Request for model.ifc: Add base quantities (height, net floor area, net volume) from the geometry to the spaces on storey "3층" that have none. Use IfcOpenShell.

First a look at what the model holds.

```python
import ifcopenshell
import ifcopenshell.util.element
import ifcopenshell.util.unit

model = ifcopenshell.open("model.ifc")
print(model.schema)
for unit_type in ("LENGTHUNIT", "AREAUNIT", "VOLUMEUNIT"):
    print(unit_type, ifcopenshell.util.unit.calculate_unit_scale(model, unit_type))
storey = next(s for s in model.by_type("IfcBuildingStorey") if s.Name == "3층")
spaces = [e for e in ifcopenshell.util.element.get_decomposition(storey) if e.is_a("IfcSpace")]
for e in sorted(spaces, key=lambda e: e.id()):
    print(e.id(), e.is_a(), e.Name, list(ifcopenshell.util.element.get_psets(e, qtos_only=True)), sep=" | ")
```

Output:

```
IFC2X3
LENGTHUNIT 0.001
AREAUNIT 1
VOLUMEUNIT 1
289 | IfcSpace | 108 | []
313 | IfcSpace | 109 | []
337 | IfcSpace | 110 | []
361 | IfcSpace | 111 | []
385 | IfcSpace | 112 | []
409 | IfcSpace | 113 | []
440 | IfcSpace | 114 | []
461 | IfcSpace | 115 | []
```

```python
import ifcopenshell
import ifcopenshell.api.pset
import ifcopenshell.geom
import ifcopenshell.util.element
import ifcopenshell.util.shape
import ifcopenshell.util.unit

model = ifcopenshell.open("model.ifc")
unit_scale = ifcopenshell.util.unit.calculate_unit_scale(model)
area_scale = ifcopenshell.util.unit.calculate_unit_scale(model, "AREAUNIT")
volume_scale = ifcopenshell.util.unit.calculate_unit_scale(model, "VOLUMEUNIT")
settings = ifcopenshell.geom.settings()

storey = next(s for s in model.by_type("IfcBuildingStorey") if s.Name == "3층")
spaces = [e for e in ifcopenshell.util.element.get_decomposition(storey) if e.is_a("IfcSpace")]

for e in sorted(spaces, key=lambda e: e.id()):
    if ifcopenshell.util.element.get_psets(e, qtos_only=True, should_inherit=False):
        continue
    # Geometry comes back in metres, in the element's own axes.
    shape = ifcopenshell.geom.create_shape(settings, e)
    values = {
        "Height": ifcopenshell.util.shape.get_z(shape.geometry) / unit_scale,
        "NetFloorArea": ifcopenshell.util.shape.get_footprint_area(shape.geometry) / area_scale,
        "NetVolume": ifcopenshell.util.shape.get_volume(shape.geometry) / volume_scale,
    }
    qto = ifcopenshell.api.pset.add_qto(model, product=e, name="BaseQuantities")
    ifcopenshell.api.pset.edit_qto(model, qto=qto, properties=values)
    print(e.id(), {k: round(v, 3) for k, v in values.items()})

model.write("model_edited.ifc")
```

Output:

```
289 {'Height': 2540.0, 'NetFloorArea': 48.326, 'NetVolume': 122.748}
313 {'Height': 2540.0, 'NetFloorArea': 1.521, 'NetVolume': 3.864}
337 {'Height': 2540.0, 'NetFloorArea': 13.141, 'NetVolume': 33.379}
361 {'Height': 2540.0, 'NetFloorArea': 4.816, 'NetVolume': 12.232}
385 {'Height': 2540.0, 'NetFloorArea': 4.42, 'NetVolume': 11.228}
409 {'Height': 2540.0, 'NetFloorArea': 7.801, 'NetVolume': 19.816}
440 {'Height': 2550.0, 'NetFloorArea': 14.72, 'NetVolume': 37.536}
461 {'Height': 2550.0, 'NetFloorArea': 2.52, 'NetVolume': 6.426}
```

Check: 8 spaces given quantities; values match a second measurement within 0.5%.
